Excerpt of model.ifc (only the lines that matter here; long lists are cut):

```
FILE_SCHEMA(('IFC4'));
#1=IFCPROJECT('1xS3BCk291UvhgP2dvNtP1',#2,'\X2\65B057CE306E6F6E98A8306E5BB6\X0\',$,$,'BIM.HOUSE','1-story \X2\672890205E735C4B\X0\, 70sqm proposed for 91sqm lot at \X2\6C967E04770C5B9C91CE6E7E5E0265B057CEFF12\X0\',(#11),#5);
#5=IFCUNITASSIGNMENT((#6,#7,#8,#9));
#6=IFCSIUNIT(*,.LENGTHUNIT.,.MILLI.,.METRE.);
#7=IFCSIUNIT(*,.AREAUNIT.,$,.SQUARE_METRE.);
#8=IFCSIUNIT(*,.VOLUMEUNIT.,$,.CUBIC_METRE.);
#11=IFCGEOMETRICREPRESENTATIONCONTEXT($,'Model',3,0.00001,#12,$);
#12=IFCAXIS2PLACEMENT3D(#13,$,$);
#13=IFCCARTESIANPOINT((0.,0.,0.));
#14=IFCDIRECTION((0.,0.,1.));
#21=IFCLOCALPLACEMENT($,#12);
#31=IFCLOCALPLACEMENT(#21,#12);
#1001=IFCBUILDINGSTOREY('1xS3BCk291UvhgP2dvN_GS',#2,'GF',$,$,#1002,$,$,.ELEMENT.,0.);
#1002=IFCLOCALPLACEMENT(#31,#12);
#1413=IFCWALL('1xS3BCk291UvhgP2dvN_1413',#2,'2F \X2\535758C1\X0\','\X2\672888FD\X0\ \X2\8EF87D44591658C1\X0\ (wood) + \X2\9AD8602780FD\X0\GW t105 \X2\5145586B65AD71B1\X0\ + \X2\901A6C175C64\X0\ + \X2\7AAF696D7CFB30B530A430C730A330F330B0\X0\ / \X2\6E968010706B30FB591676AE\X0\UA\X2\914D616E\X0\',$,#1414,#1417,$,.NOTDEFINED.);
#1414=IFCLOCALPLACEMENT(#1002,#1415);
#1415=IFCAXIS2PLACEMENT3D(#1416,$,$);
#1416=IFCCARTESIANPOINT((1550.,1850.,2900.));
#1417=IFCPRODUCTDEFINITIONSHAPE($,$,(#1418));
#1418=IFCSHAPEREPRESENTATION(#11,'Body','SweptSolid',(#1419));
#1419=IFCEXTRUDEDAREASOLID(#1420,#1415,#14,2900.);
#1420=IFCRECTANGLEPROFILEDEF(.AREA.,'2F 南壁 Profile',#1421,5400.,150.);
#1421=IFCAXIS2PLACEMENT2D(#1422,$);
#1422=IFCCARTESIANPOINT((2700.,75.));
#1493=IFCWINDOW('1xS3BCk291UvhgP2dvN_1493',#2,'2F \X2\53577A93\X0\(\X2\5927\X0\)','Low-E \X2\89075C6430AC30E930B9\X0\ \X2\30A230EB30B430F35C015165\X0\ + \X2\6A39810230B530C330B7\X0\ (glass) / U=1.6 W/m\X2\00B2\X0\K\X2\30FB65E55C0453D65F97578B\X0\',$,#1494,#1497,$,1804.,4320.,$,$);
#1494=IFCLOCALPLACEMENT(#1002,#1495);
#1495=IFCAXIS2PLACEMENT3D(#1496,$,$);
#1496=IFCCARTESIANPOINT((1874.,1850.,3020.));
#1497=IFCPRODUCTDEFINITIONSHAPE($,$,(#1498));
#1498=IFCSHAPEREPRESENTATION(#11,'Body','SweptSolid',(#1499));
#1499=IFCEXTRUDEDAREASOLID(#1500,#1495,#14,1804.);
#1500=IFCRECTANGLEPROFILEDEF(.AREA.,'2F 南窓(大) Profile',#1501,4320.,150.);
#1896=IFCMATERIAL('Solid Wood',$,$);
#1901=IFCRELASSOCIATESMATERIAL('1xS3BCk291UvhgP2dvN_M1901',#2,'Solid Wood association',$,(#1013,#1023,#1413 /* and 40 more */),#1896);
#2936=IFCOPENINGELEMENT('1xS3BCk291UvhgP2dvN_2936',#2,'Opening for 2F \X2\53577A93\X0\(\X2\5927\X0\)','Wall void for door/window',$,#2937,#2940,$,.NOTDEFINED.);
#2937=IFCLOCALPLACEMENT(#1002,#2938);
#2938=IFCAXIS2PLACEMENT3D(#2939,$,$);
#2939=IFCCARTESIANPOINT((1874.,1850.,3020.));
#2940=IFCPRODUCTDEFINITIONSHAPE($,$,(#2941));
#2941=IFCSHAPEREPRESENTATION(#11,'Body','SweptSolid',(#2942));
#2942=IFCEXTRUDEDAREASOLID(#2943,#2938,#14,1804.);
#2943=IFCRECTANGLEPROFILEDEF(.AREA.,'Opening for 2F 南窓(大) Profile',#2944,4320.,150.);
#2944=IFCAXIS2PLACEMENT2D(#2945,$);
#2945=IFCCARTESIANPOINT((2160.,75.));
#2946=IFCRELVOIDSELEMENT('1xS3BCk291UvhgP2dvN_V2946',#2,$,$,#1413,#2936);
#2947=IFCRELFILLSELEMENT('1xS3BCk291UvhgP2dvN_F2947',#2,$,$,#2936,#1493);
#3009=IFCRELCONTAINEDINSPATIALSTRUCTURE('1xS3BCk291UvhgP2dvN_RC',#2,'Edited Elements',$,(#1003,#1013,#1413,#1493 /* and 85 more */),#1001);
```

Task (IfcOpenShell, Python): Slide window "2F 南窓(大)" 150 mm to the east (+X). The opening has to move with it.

```python
import ifcopenshell
import ifcopenshell.api.geometry
import ifcopenshell.util.placement
import ifcopenshell.util.unit

model = ifcopenshell.open("model.ifc")
unit_scale = ifcopenshell.util.unit.calculate_unit_scale(model)

window = model.by_guid("1xS3BCk291UvhgP2dvN_1493")
opening = window.FillsVoids[0].RelatingOpeningElement
wall = opening.VoidsElements[0].RelatingBuildingElement

wall_matrix = ifcopenshell.util.placement.get_local_placement(wall.ObjectPlacement)
shift = wall_matrix[:3, 0] * 0.15 / unit_scale
before = ifcopenshell.util.placement.get_local_placement(window.ObjectPlacement)[:3, 3].copy()

# The window is not placed relative to its opening, so move both.
for product in (opening, window):
    matrix = ifcopenshell.util.placement.get_local_placement(product.ObjectPlacement)
    matrix[:3, 3] += shift
    ifcopenshell.api.geometry.edit_object_placement(model, product=product, matrix=matrix, is_si=False)

after = ifcopenshell.util.placement.get_local_placement(window.ObjectPlacement)[:3, 3]
print("window moved by", (after - before).round(3) + 0.0)

model.write("model_rev.ifc")
```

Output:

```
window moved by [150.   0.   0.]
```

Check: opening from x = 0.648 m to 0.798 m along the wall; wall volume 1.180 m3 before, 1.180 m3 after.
